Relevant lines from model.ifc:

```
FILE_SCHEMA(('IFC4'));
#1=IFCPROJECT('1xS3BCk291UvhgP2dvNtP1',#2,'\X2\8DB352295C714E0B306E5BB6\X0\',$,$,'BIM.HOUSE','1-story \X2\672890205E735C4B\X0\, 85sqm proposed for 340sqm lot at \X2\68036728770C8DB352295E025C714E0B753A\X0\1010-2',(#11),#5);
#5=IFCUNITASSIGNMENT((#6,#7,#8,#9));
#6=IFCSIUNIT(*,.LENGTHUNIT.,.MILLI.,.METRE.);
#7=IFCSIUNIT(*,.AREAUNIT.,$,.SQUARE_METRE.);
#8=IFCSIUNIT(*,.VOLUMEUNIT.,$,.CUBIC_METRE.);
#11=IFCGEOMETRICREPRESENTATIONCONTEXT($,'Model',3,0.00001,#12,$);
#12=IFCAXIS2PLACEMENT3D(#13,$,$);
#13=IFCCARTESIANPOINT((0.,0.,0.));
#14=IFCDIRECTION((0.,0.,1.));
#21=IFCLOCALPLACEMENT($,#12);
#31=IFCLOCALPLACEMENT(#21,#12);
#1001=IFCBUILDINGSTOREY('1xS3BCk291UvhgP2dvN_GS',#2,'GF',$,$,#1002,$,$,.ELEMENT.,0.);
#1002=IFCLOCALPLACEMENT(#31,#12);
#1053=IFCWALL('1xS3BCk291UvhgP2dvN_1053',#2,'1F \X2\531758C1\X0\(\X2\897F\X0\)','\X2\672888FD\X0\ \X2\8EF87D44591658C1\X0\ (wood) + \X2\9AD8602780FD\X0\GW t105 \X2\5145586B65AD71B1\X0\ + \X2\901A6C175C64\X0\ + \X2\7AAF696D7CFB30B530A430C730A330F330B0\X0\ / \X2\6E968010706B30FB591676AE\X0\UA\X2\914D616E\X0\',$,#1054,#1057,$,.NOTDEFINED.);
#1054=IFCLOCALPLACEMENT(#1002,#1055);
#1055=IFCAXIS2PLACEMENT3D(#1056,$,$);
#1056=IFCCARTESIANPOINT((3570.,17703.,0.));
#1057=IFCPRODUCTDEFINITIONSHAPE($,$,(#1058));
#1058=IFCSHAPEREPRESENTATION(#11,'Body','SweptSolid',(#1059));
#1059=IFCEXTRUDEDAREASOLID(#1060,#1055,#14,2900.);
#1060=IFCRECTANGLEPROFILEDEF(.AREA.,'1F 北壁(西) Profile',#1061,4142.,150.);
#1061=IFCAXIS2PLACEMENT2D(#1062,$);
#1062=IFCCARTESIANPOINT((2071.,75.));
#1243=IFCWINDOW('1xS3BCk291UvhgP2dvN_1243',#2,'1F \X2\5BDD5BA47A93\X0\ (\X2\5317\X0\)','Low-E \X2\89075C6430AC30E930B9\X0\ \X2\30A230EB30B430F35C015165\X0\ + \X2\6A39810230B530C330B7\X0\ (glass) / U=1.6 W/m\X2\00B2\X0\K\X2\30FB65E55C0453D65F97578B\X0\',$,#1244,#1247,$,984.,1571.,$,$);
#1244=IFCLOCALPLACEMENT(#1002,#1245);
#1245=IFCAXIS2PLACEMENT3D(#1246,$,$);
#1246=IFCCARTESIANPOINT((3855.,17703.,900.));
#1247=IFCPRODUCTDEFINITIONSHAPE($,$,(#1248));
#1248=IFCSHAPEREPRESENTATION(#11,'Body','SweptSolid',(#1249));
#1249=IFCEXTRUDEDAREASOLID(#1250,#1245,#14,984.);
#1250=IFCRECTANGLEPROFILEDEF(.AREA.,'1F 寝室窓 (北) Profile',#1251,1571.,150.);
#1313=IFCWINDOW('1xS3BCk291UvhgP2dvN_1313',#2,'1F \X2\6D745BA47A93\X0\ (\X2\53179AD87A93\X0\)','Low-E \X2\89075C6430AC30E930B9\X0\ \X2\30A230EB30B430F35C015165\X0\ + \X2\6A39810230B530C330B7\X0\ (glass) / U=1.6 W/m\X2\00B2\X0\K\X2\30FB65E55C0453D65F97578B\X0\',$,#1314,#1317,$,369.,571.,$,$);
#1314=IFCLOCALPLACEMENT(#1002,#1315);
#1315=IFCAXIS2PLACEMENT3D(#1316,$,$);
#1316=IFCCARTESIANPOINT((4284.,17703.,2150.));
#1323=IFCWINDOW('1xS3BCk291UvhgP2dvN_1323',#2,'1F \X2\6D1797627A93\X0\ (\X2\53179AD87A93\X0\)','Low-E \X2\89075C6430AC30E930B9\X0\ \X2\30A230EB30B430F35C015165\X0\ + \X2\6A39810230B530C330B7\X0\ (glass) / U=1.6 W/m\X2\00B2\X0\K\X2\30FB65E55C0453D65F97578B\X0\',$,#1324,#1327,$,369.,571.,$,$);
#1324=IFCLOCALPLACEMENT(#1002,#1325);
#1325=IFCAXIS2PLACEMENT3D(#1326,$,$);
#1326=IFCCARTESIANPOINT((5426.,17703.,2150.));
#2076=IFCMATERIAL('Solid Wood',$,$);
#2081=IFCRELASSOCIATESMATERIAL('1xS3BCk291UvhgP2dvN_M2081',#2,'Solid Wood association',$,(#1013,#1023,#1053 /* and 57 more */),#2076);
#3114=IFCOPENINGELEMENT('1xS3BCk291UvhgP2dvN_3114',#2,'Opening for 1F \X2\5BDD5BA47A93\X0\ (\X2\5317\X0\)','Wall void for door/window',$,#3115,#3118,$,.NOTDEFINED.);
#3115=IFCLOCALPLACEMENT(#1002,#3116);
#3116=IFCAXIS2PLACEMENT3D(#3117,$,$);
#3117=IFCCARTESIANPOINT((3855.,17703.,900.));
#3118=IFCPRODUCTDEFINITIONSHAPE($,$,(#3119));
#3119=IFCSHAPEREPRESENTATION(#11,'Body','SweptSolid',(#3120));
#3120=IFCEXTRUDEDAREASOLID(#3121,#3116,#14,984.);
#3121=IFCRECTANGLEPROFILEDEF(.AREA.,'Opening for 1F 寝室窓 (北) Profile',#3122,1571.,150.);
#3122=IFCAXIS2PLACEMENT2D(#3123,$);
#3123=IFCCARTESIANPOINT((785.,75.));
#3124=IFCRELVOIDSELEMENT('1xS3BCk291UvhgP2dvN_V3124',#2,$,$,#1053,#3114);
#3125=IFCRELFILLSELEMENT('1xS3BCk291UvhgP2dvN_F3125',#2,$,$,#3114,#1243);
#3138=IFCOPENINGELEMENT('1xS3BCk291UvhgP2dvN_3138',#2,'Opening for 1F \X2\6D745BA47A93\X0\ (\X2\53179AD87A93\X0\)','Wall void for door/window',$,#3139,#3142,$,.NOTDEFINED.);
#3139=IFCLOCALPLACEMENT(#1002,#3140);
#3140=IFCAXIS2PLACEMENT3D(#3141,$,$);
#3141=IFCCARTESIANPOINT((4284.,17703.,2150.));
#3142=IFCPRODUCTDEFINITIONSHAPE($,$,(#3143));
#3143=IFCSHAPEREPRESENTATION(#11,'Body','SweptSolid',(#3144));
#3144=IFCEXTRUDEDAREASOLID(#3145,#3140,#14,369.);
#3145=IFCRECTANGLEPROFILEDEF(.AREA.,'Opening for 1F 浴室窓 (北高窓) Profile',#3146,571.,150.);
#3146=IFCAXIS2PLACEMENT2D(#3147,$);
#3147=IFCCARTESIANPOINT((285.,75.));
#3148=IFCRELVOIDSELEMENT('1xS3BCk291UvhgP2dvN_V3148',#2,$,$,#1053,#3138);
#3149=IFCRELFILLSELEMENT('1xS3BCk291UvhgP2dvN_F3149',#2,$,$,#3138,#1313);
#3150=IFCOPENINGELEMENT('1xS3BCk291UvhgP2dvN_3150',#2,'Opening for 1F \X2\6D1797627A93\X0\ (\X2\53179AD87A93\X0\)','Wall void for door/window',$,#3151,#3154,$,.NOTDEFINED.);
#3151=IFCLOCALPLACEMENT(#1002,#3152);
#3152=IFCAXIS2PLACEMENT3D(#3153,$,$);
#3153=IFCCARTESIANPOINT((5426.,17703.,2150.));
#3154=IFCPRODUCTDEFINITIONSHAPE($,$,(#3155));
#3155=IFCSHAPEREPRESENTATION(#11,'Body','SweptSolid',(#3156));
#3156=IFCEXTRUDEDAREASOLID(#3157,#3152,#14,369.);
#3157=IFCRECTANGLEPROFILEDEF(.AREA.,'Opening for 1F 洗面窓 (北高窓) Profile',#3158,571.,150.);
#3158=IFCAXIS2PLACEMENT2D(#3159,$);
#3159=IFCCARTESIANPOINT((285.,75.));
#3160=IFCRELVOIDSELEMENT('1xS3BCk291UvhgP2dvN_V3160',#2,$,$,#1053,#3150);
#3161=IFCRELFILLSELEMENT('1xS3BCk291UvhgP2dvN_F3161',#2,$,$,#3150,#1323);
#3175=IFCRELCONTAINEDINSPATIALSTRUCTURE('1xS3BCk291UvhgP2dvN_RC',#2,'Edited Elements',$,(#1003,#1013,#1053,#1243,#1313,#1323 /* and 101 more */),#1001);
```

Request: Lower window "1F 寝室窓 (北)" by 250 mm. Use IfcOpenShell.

```python
import numpy as np
import ifcopenshell
import ifcopenshell.api.geometry
import ifcopenshell.util.placement
import ifcopenshell.util.unit

model = ifcopenshell.open("model.ifc")
unit_scale = ifcopenshell.util.unit.calculate_unit_scale(model)

window = model.by_id(1243)
opening = window.FillsVoids[0].RelatingOpeningElement
dz = -250.0

shift = np.array([0.0, 0.0, dz])
# The window is not placed relative to its opening, so move both.
for product in (opening, window):
    matrix = ifcopenshell.util.placement.get_local_placement(product.ObjectPlacement)
    matrix[:3, 3] += shift
    ifcopenshell.api.geometry.edit_object_placement(model, product=product, matrix=matrix, is_si=False)

print(f"moved by {dz * unit_scale:+.3f} m")

model.write("model_rev.ifc")
```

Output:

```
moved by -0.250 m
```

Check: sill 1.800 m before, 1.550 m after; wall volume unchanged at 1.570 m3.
